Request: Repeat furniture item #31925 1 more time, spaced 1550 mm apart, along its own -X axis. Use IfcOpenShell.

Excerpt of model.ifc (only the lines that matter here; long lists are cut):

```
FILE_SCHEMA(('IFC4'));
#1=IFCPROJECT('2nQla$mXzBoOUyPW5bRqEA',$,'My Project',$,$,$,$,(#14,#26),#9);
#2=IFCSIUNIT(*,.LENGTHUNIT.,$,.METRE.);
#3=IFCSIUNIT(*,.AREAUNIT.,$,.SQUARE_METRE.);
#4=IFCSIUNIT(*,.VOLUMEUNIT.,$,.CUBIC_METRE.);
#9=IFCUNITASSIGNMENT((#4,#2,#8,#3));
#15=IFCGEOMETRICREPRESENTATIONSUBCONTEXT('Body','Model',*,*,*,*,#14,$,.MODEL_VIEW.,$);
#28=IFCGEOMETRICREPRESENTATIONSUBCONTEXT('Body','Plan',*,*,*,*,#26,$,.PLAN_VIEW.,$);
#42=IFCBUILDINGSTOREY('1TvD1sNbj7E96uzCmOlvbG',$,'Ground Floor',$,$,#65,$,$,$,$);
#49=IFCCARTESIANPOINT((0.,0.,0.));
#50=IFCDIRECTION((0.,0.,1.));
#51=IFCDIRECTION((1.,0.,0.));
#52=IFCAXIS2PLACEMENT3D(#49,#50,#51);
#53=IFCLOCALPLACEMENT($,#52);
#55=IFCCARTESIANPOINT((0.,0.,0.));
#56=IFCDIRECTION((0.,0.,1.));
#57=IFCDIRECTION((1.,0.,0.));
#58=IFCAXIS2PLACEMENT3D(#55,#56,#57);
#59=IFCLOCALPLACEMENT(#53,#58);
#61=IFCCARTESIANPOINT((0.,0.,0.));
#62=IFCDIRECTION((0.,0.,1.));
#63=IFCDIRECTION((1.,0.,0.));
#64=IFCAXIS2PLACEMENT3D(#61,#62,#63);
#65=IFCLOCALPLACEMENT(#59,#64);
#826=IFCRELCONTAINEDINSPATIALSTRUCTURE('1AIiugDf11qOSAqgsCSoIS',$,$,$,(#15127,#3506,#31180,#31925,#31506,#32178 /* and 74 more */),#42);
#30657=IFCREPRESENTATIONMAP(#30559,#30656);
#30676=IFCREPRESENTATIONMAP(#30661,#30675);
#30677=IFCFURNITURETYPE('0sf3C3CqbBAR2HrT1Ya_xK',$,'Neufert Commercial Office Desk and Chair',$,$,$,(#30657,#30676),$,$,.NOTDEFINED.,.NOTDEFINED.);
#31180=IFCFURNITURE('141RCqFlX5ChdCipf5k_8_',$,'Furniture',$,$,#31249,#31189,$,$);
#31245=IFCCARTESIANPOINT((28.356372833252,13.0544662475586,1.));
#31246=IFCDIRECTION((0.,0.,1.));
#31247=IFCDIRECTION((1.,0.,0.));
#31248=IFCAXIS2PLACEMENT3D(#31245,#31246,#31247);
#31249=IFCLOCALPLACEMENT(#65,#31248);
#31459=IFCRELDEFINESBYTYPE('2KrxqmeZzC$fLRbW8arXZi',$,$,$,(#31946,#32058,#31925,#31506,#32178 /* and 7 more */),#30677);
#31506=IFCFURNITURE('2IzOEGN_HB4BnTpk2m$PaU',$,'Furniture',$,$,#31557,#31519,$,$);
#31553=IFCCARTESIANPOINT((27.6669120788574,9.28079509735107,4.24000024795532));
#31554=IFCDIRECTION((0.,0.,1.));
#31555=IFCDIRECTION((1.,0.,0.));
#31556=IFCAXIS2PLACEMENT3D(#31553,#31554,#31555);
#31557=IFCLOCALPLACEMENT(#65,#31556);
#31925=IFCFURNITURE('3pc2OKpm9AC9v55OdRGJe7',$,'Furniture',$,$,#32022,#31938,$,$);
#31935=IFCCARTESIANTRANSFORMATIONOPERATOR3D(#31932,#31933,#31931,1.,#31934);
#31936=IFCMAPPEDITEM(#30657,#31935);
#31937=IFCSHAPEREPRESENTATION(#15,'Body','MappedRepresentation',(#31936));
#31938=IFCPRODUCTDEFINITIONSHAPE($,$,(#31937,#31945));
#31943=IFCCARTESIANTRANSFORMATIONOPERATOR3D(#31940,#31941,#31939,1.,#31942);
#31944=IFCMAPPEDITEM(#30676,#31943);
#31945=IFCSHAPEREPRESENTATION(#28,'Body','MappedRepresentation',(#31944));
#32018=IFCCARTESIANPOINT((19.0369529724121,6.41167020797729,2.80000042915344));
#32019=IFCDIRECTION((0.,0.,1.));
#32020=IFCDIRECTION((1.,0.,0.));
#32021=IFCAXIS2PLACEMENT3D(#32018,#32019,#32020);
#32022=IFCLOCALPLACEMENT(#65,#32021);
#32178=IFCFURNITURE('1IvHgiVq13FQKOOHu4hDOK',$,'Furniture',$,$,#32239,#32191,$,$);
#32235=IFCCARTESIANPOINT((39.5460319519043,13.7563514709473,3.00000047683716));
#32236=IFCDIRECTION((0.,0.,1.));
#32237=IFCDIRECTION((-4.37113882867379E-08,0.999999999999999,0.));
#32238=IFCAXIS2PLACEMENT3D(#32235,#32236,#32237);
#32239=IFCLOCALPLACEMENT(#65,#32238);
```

```python
import ifcopenshell
import ifcopenshell.api.geometry
import ifcopenshell.api.root
import ifcopenshell.util.element
import ifcopenshell.util.placement

model = ifcopenshell.open("model.ifc")

source = model.by_guid("3pc2OKpm9AC9v55OdRGJe7")
base = ifcopenshell.util.placement.get_local_placement(source.ObjectPlacement)
step = -base[:3, 0] * 1.55

for i in range(1, 2):
    copy = ifcopenshell.api.root.copy_class(model, product=source)
    copy.Representation = ifcopenshell.util.element.copy_deep(
        model, source.Representation, exclude=["IfcGeometricRepresentationContext", "IfcRepresentationMap"]
    )
    matrix = base.copy()
    matrix[:3, 3] += i * step
    print("added at", matrix[:3, 3].round(3) + 0.0)
    ifcopenshell.api.geometry.edit_object_placement(model, product=copy, matrix=matrix, is_si=False)

model.write("model_edited.ifc")
```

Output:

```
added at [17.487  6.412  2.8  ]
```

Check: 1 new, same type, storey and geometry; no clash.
